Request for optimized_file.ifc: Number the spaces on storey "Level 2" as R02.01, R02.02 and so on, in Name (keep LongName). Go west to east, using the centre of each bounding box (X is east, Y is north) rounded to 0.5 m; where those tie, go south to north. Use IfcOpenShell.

First a look at what the model holds.

```python
import ifcopenshell
import ifcopenshell.util.element
import ifcopenshell.util.placement

model = ifcopenshell.open("optimized_file.ifc")
print(model.schema)
storey = next(s for s in model.by_type("IfcBuildingStorey") if s.Name == "Level 2")
spaces = [e for e in ifcopenshell.util.element.get_decomposition(storey) if e.is_a("IfcSpace")]
for e in sorted(spaces, key=lambda e: e.id()):
    origin = ifcopenshell.util.placement.get_local_placement(e.ObjectPlacement)[:3, 3]
    print(e.id(), e.Name, e.LongName, origin.round(2) + 0.0, sep=" | ")
```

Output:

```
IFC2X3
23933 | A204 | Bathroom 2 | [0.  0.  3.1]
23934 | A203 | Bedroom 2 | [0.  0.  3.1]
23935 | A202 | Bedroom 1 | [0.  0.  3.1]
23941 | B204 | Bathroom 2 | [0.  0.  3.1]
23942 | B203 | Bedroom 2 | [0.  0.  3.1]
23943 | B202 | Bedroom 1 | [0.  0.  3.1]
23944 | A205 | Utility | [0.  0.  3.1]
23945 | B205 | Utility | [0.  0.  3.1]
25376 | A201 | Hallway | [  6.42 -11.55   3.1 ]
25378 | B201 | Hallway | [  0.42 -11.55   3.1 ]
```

```python
import ifcopenshell
import ifcopenshell.geom
import ifcopenshell.util.element
import ifcopenshell.util.shape

model = ifcopenshell.open("optimized_file.ifc")
settings = ifcopenshell.geom.settings()
settings.set("use-world-coords", True)


def centre(element):
    shape = ifcopenshell.geom.create_shape(settings, element)
    return ifcopenshell.util.shape.get_bbox_centroid(shape.geometry)


storey = next(s for s in model.by_type("IfcBuildingStorey") if s.Name == "Level 2")
spaces = [e for e in ifcopenshell.util.element.get_decomposition(storey) if e.is_a("IfcSpace")]

# Insertion points can sit at a corner or the storey origin, so sort by the geometry (in metres).
centres = {e: centre(e) for e in spaces}
spaces.sort(key=lambda e: (round(centres[e][0] / 0.5), centres[e][1]))

for i, e in enumerate(spaces, start=1):
    number = f"R02.{i:02d}"
    e.Name = number
    print(e.id(), number)

model.write("optimized_file_edited.ifc")
```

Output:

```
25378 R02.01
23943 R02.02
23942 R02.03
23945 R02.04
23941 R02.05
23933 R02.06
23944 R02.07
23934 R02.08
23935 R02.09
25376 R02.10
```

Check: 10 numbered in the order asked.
